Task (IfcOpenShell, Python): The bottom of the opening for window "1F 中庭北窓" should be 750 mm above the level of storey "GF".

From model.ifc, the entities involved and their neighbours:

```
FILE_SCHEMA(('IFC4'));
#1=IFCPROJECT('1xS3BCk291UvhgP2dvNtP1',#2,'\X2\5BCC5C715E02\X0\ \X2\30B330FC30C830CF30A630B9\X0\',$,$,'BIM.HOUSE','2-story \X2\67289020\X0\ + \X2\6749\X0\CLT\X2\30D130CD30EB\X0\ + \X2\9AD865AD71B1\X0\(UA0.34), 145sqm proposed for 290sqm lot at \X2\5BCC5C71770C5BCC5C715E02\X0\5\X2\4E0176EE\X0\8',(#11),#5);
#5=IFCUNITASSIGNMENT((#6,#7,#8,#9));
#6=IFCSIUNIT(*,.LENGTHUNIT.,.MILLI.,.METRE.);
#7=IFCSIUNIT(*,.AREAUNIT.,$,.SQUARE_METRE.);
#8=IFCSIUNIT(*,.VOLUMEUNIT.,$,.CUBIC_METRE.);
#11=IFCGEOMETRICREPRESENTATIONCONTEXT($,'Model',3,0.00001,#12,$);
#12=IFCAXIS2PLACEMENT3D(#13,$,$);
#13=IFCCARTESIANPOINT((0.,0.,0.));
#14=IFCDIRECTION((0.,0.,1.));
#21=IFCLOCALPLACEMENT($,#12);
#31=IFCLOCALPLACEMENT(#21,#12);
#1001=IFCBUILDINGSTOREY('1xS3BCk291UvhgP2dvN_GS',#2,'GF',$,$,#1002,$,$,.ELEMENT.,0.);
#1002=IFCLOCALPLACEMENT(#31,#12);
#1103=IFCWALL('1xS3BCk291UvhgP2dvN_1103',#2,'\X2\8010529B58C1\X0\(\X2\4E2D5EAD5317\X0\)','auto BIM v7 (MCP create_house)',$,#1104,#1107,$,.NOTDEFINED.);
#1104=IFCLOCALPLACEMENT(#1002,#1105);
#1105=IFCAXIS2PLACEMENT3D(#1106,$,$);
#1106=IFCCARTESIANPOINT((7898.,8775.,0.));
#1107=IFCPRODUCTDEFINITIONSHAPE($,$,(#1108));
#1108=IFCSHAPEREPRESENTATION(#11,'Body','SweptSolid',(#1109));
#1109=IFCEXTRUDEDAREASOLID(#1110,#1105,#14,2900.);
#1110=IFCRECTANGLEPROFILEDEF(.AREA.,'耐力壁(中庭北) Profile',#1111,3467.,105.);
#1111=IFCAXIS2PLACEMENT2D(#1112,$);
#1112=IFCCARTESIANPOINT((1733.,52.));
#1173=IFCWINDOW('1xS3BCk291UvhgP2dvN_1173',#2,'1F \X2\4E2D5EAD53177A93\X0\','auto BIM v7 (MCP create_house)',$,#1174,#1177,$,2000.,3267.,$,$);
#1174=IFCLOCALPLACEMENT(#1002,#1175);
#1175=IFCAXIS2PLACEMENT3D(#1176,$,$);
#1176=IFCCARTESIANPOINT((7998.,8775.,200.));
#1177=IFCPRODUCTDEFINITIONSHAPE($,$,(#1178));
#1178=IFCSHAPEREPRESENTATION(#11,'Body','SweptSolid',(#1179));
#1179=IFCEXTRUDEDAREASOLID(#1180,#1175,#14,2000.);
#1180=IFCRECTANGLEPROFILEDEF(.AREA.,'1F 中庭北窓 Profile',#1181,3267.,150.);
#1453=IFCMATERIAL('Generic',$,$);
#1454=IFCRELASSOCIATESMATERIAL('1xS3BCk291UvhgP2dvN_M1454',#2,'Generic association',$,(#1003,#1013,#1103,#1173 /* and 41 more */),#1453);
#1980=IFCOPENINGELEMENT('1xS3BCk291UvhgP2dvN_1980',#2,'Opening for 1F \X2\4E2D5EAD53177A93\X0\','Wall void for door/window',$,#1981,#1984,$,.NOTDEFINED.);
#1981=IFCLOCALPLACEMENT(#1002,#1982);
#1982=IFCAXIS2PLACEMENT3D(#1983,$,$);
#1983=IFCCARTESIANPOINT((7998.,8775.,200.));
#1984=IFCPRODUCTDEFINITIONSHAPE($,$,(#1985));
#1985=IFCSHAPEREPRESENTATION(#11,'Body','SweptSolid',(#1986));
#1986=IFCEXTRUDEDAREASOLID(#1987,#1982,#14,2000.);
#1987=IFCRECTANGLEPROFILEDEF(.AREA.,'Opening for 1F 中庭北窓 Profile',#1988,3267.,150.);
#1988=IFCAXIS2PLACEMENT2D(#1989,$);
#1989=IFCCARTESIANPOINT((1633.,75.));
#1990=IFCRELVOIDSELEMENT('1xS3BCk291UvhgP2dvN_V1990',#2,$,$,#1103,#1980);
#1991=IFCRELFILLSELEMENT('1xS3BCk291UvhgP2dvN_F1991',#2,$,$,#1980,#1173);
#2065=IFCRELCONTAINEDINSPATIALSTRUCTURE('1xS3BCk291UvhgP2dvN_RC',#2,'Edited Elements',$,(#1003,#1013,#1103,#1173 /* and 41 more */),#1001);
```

```python
import numpy as np
import ifcopenshell
import ifcopenshell.api.geometry
import ifcopenshell.geom
import ifcopenshell.util.element
import ifcopenshell.util.placement
import ifcopenshell.util.shape
import ifcopenshell.util.unit

model = ifcopenshell.open("model.ifc")
unit_scale = ifcopenshell.util.unit.calculate_unit_scale(model)

window = model.by_id(1173)
opening = window.FillsVoids[0].RelatingOpeningElement
storey = ifcopenshell.util.element.get_container(window, ifc_class="IfcBuildingStorey")
level = ifcopenshell.util.placement.get_local_placement(storey.ObjectPlacement)[2, 3]

# The opening's origin need not be at the sill, so measure its lowest point.
shape = ifcopenshell.geom.create_shape(ifcopenshell.geom.settings(), opening)
bottom = ifcopenshell.util.shape.get_shape_bottom_elevation(shape, shape.geometry) / unit_scale
dz = level + 0.75 / unit_scale - bottom

shift = np.array([0.0, 0.0, dz])
# The window is not placed relative to its opening, so move both.
for product in (opening, window):
    matrix = ifcopenshell.util.placement.get_local_placement(product.ObjectPlacement)
    matrix[:3, 3] += shift
    ifcopenshell.api.geometry.edit_object_placement(model, product=product, matrix=matrix, is_si=False)

print(f"moved by {dz * unit_scale:+.3f} m")

model.write("model_updated.ifc")
```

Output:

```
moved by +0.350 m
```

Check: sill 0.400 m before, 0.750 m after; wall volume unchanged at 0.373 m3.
